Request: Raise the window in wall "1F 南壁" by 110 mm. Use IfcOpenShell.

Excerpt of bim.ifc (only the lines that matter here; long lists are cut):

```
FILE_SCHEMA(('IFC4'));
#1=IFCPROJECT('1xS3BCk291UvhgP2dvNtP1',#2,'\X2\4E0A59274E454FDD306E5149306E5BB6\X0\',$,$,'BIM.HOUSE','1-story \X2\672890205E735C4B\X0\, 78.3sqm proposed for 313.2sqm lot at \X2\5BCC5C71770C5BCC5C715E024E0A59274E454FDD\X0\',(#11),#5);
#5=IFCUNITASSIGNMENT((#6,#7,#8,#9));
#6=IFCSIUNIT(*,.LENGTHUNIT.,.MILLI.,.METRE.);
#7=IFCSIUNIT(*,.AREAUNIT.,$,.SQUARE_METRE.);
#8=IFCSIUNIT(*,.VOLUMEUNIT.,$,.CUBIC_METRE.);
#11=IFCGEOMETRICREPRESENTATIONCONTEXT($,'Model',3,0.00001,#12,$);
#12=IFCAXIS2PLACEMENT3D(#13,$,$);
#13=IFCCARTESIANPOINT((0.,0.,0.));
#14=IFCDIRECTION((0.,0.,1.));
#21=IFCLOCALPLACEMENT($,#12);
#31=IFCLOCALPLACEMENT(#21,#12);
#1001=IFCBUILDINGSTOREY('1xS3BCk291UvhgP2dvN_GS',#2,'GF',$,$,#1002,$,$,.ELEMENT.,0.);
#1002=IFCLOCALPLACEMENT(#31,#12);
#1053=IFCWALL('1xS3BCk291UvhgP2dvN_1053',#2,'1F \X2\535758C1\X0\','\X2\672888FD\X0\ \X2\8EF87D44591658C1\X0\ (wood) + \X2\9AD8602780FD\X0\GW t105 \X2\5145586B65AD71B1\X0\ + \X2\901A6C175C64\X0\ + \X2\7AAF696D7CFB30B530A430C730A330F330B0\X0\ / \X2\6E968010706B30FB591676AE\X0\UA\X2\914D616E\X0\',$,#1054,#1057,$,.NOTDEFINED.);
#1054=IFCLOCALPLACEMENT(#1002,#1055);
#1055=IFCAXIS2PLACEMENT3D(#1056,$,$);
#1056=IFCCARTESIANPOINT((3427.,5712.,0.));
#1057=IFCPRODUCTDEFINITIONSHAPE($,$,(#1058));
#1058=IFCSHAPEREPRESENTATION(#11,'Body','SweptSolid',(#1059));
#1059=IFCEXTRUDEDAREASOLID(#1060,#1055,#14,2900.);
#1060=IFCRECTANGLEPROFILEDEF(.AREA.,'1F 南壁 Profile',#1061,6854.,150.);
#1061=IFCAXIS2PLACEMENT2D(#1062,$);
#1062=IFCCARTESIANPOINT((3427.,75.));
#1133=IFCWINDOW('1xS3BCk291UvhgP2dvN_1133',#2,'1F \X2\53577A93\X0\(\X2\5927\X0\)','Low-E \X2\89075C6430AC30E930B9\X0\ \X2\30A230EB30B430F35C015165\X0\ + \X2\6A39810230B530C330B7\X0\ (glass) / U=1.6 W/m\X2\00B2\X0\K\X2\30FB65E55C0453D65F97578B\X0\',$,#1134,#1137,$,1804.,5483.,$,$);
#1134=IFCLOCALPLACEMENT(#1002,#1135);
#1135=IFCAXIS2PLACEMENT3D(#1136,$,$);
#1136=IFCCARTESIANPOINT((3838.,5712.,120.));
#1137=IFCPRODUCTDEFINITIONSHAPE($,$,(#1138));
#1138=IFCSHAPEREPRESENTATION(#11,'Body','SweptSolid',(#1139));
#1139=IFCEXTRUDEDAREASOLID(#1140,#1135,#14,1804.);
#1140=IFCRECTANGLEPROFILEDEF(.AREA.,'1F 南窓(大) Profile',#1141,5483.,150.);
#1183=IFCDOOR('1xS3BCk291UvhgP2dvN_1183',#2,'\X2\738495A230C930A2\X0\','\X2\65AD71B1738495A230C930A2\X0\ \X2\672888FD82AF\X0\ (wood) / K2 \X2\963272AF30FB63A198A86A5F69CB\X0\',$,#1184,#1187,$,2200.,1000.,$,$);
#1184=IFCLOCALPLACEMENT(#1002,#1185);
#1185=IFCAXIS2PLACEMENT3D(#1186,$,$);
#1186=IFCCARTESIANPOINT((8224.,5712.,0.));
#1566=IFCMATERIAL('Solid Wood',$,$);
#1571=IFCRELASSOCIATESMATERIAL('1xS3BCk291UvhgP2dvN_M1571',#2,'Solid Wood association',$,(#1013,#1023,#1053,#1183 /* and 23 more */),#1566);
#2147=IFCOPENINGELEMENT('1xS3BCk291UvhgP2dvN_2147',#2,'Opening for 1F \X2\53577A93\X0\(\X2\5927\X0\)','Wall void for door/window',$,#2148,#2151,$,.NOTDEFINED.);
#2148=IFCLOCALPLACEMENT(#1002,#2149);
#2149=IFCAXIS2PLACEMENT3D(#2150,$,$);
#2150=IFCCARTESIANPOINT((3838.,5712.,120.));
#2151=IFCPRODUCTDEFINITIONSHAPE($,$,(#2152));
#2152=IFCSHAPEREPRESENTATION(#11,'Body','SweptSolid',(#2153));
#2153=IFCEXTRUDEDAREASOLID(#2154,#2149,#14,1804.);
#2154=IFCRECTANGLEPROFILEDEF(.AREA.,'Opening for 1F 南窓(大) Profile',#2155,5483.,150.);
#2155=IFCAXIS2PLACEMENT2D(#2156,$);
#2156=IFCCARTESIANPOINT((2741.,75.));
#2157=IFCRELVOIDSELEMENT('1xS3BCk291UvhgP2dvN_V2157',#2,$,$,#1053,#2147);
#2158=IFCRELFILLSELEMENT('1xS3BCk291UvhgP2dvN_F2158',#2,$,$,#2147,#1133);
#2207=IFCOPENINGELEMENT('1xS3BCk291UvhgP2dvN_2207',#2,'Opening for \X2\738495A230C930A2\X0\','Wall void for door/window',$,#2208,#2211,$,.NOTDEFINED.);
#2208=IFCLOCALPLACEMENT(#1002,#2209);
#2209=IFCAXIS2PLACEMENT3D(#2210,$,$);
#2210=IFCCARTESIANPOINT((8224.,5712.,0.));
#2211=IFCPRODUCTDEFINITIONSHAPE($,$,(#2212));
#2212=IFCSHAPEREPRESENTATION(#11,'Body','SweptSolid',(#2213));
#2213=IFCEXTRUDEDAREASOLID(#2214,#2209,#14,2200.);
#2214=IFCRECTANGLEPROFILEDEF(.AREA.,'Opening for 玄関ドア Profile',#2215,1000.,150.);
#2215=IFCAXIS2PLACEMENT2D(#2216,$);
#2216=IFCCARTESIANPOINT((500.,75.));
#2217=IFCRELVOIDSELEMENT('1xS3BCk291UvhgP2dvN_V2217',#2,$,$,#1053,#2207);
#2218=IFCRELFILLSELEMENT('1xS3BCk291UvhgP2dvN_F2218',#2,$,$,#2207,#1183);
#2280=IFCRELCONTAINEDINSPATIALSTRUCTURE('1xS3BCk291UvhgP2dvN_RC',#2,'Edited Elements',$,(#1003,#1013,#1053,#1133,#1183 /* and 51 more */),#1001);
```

```python
import numpy as np
import ifcopenshell
import ifcopenshell.api.geometry
import ifcopenshell.util.placement
import ifcopenshell.util.unit

model = ifcopenshell.open("bim.ifc")
unit_scale = ifcopenshell.util.unit.calculate_unit_scale(model)

window = model.by_guid("1xS3BCk291UvhgP2dvN_1133")
opening = window.FillsVoids[0].RelatingOpeningElement
dz = 110.0

shift = np.array([0.0, 0.0, dz])
# The window is not placed relative to its opening, so move both.
for product in (opening, window):
    matrix = ifcopenshell.util.placement.get_local_placement(product.ObjectPlacement)
    matrix[:3, 3] += shift
    ifcopenshell.api.geometry.edit_object_placement(model, product=product, matrix=matrix, is_si=False)

print(f"moved by {dz * unit_scale:+.3f} m")

model.write("bim_rev.ifc")
```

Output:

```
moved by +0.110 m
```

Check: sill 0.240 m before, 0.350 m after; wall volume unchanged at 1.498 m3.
